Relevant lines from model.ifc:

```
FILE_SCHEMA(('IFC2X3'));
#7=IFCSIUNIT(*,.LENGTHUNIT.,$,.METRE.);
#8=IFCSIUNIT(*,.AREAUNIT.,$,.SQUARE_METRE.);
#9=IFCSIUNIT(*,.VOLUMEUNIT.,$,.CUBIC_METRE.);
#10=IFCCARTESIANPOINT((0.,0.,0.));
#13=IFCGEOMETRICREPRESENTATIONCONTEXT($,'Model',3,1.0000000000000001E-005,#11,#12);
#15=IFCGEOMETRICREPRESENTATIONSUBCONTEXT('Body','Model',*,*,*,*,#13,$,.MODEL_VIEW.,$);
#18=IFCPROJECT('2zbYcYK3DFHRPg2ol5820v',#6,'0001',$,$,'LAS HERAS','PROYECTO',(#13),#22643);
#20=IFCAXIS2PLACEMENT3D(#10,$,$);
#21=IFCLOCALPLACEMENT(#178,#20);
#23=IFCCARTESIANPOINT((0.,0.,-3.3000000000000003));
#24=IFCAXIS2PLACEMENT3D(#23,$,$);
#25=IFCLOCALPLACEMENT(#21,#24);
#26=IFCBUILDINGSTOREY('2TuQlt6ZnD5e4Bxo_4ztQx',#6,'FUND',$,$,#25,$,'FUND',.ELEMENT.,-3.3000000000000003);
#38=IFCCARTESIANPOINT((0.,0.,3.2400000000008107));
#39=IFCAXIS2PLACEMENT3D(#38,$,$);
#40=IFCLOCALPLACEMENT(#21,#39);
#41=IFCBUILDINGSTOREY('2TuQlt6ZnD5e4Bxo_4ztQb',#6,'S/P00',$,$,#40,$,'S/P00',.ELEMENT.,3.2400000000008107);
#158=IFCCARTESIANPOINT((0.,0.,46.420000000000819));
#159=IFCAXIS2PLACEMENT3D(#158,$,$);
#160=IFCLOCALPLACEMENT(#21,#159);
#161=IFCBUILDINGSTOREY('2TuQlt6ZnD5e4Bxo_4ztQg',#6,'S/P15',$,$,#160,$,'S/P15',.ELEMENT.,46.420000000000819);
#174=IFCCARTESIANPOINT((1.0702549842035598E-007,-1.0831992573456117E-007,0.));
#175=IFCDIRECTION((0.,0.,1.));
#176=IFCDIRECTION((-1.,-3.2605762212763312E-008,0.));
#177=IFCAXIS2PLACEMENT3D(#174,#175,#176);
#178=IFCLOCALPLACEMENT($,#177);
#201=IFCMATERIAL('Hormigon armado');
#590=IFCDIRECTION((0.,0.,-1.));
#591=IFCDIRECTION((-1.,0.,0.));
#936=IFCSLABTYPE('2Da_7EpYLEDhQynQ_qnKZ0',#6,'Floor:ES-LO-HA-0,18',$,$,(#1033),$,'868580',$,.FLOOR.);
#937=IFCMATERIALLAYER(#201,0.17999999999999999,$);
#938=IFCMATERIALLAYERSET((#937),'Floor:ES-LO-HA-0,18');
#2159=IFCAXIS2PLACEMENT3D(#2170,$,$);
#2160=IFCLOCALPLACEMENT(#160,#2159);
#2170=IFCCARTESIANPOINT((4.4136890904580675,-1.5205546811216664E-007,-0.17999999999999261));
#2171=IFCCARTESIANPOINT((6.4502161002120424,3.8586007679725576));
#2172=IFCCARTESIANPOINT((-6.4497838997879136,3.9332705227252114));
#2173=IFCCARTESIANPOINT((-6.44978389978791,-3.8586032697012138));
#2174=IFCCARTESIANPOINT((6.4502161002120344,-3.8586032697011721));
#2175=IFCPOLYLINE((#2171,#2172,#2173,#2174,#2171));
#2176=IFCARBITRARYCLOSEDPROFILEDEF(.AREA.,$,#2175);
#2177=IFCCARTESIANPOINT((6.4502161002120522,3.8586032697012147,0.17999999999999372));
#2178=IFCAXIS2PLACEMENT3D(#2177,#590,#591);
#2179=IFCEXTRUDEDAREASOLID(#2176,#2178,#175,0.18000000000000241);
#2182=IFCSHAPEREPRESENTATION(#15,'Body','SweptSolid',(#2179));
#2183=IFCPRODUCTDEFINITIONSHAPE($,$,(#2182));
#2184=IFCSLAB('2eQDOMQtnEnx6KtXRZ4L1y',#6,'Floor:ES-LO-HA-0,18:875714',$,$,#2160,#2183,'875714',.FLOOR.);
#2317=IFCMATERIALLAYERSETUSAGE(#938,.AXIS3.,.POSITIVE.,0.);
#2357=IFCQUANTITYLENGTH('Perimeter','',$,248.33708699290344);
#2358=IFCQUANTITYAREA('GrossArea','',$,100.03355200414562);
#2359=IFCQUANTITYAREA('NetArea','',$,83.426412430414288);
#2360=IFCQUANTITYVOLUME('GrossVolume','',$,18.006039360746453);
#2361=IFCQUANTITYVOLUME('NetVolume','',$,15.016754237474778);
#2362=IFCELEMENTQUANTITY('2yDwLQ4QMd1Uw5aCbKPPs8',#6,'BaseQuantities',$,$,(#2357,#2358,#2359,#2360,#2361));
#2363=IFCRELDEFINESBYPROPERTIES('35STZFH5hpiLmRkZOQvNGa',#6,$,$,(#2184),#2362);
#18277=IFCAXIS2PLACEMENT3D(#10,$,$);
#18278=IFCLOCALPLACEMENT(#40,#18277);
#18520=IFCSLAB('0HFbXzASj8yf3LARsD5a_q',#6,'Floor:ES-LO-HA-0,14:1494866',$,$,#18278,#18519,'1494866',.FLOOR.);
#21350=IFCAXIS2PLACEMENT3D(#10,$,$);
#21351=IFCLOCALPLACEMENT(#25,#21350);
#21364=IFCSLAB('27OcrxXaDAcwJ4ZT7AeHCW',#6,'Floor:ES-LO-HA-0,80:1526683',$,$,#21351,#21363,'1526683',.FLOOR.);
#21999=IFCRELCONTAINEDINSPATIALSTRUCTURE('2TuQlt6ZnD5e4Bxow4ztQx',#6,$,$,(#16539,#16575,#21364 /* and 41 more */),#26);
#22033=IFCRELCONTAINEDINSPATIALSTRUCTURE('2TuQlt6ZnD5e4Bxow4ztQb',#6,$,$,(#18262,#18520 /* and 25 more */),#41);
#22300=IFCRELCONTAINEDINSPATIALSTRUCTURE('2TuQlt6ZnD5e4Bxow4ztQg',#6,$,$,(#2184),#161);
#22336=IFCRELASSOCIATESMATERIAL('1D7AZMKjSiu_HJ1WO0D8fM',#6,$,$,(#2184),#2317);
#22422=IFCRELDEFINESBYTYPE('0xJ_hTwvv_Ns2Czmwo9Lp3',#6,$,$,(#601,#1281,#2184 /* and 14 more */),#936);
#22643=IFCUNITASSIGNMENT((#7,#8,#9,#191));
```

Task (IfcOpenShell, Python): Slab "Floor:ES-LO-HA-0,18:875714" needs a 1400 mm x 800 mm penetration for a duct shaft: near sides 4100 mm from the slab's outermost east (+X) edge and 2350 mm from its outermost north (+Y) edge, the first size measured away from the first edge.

```python
import numpy as np
import ifcopenshell
import ifcopenshell.api.feature
import ifcopenshell.api.geometry
import ifcopenshell.api.pset
import ifcopenshell.api.root
import ifcopenshell.geom
import ifcopenshell.util.element
import ifcopenshell.util.placement
import ifcopenshell.util.representation
import ifcopenshell.util.shape
import ifcopenshell.util.unit

model = ifcopenshell.open("model.ifc")
unit_scale = ifcopenshell.util.unit.calculate_unit_scale(model)
area_scale = ifcopenshell.util.unit.calculate_unit_scale(model, "AREAUNIT")
volume_scale = ifcopenshell.util.unit.calculate_unit_scale(model, "VOLUMEUNIT")
settings = ifcopenshell.geom.settings()


def volume(element):
    """Net volume in cubic metres, openings subtracted."""
    shape = ifcopenshell.geom.create_shape(settings, element)
    return ifcopenshell.util.shape.get_volume(shape.geometry)


slab = model.by_guid("2eQDOMQtnEnx6KtXRZ4L1y")
before = volume(slab)

# Extent in the slab's own axes, in metres. The edges named are its -X and -Y sides.
slab_shape = ifcopenshell.geom.create_shape(settings, slab)
vertices = ifcopenshell.util.shape.get_vertices(slab_shape.geometry)
x_min, y_min, bottom = vertices.min(axis=0)
top = vertices[:, 2].max()

opening = ifcopenshell.api.root.create_entity(model, ifc_class="IfcOpeningElement", name="Duct shaft opening")
context = ifcopenshell.util.representation.get_context(model, "Model", "Body", "MODEL_VIEW")
width, depth = 1.4, 0.8
outline = [(0.0, 0.0), (width, 0.0), (width, depth), (0.0, depth), (0.0, 0.0)]
# Overshoot both faces by 50 mm so the cut is clean.
shape = ifcopenshell.api.geometry.add_slab_representation(
    model, context=context, depth=top - bottom + 0.1, polyline=outline
)
ifcopenshell.api.geometry.assign_representation(model, product=opening, representation=shape)

matrix = ifcopenshell.util.placement.get_local_placement(slab.ObjectPlacement)
matrix[:, 3] = matrix @ np.append(np.array([x_min + 4.1, y_min + 2.35, bottom - 0.05]) / unit_scale, 1.0)
ifcopenshell.api.geometry.edit_object_placement(model, product=opening, matrix=matrix, is_si=False)
ifcopenshell.api.feature.add_feature(model, feature=opening, element=slab)

after = volume(slab)

# Update the slab's stored quantities.
qto = model.by_id(ifcopenshell.util.element.get_pset(slab, "BaseQuantities", should_inherit=False)["id"])
ifcopenshell.api.pset.edit_qto(model, qto=qto, properties={
    "NetArea": after / (top - bottom) / area_scale,
    "NetVolume": after / volume_scale,
})

print(f"slab volume {before:.3f} -> {after:.3f} m3")

model.write("model_updated.ifc")
```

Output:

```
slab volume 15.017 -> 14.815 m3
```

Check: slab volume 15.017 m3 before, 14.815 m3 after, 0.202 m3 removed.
